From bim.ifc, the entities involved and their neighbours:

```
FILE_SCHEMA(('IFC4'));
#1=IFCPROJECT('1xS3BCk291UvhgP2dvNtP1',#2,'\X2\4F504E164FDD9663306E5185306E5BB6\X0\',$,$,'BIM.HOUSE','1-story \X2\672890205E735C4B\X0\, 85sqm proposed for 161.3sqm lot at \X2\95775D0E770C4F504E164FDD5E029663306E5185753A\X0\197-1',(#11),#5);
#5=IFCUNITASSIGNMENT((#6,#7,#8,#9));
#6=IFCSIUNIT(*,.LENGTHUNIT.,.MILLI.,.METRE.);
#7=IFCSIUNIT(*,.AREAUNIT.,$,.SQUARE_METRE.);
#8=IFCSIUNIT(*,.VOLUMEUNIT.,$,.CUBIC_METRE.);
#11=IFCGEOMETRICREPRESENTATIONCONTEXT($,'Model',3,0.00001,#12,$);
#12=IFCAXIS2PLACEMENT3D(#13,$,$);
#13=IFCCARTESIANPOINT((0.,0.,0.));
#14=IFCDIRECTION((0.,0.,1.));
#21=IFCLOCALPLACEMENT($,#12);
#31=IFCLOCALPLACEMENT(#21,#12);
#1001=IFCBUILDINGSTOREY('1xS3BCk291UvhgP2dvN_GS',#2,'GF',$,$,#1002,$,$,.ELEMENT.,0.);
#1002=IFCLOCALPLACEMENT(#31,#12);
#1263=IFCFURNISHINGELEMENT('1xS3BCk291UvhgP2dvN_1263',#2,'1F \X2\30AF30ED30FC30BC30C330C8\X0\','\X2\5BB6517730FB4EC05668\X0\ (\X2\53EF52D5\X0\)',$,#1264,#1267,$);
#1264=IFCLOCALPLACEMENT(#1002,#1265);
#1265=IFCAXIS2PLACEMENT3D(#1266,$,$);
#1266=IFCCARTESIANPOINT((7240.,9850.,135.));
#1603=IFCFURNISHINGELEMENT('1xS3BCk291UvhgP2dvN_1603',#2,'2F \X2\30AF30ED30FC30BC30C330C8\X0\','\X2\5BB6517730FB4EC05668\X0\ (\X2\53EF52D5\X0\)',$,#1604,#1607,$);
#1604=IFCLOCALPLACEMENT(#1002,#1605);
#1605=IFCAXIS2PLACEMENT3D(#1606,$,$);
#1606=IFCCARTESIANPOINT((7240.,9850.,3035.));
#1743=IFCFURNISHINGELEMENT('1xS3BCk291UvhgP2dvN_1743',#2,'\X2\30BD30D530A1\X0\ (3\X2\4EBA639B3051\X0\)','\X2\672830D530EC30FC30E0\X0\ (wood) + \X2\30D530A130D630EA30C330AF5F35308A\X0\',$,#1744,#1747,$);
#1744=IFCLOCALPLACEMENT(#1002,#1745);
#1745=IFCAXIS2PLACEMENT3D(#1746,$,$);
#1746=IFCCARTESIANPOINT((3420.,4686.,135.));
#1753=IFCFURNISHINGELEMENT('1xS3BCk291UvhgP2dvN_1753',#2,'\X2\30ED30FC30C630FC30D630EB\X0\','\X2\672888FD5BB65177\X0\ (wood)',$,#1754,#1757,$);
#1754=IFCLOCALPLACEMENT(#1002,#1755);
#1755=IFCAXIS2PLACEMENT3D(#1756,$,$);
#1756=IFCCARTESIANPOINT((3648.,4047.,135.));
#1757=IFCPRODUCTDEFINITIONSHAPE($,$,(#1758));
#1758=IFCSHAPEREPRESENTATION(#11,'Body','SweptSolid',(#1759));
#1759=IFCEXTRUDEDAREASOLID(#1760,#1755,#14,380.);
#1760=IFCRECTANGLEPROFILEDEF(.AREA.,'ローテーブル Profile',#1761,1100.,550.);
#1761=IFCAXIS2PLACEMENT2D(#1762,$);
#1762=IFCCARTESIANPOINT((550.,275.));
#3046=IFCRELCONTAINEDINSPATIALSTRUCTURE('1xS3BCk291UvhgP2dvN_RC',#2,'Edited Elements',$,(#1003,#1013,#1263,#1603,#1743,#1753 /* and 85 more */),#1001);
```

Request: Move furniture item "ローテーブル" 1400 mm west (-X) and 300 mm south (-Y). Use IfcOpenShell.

```python
import ifcopenshell
import ifcopenshell.api.geometry
import ifcopenshell.util.placement
import ifcopenshell.util.unit

model = ifcopenshell.open("bim.ifc")
unit_scale = ifcopenshell.util.unit.calculate_unit_scale(model)

item = model.by_guid("1xS3BCk291UvhgP2dvN_1753")
matrix = ifcopenshell.util.placement.get_local_placement(item.ObjectPlacement)
matrix[0, 3] -= 1.4 / unit_scale
matrix[1, 3] -= 0.3 / unit_scale
ifcopenshell.api.geometry.edit_object_placement(model, product=item, matrix=matrix, is_si=False)

print(ifcopenshell.util.placement.get_local_placement(item.ObjectPlacement).round(3) + 0.0)

model.write("bim_v2.ifc")
```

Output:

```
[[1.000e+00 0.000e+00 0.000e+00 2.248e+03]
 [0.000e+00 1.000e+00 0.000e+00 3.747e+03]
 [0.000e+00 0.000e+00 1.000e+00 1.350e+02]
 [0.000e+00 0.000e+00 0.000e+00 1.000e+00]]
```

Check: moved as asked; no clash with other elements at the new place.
